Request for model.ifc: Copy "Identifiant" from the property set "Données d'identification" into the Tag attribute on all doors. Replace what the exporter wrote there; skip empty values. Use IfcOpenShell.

First a look at what the model holds.

```python
import ifcopenshell
import ifcopenshell.util.element

model = ifcopenshell.open("model.ifc")
print(model.schema)
doors = model.by_type("IfcDoor")
print(len(doors), "doors")
for e in doors[:8]:
    source = ifcopenshell.util.element.get_pset(e, "Données d'identification", "Identifiant")
    target = e.Tag
    print(e.id(), repr(source), repr(target), sep=" | ")
```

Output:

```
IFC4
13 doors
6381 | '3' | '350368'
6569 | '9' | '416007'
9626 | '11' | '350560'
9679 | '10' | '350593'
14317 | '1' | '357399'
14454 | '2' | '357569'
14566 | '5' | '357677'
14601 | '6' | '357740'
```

```python
import ifcopenshell
import ifcopenshell.util.element

model = ifcopenshell.open("model.ifc")

count = 0
for e in model.by_type("IfcDoor"):
    value = ifcopenshell.util.element.get_pset(e, "Données d'identification", "Identifiant")
    current = e.Tag
    if not value or not value.strip() or current == value:
        continue
    e.Tag = value
    count += 1

print(count, "doors updated")

model.write("model_v2.ifc")
```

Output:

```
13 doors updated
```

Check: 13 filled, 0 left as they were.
